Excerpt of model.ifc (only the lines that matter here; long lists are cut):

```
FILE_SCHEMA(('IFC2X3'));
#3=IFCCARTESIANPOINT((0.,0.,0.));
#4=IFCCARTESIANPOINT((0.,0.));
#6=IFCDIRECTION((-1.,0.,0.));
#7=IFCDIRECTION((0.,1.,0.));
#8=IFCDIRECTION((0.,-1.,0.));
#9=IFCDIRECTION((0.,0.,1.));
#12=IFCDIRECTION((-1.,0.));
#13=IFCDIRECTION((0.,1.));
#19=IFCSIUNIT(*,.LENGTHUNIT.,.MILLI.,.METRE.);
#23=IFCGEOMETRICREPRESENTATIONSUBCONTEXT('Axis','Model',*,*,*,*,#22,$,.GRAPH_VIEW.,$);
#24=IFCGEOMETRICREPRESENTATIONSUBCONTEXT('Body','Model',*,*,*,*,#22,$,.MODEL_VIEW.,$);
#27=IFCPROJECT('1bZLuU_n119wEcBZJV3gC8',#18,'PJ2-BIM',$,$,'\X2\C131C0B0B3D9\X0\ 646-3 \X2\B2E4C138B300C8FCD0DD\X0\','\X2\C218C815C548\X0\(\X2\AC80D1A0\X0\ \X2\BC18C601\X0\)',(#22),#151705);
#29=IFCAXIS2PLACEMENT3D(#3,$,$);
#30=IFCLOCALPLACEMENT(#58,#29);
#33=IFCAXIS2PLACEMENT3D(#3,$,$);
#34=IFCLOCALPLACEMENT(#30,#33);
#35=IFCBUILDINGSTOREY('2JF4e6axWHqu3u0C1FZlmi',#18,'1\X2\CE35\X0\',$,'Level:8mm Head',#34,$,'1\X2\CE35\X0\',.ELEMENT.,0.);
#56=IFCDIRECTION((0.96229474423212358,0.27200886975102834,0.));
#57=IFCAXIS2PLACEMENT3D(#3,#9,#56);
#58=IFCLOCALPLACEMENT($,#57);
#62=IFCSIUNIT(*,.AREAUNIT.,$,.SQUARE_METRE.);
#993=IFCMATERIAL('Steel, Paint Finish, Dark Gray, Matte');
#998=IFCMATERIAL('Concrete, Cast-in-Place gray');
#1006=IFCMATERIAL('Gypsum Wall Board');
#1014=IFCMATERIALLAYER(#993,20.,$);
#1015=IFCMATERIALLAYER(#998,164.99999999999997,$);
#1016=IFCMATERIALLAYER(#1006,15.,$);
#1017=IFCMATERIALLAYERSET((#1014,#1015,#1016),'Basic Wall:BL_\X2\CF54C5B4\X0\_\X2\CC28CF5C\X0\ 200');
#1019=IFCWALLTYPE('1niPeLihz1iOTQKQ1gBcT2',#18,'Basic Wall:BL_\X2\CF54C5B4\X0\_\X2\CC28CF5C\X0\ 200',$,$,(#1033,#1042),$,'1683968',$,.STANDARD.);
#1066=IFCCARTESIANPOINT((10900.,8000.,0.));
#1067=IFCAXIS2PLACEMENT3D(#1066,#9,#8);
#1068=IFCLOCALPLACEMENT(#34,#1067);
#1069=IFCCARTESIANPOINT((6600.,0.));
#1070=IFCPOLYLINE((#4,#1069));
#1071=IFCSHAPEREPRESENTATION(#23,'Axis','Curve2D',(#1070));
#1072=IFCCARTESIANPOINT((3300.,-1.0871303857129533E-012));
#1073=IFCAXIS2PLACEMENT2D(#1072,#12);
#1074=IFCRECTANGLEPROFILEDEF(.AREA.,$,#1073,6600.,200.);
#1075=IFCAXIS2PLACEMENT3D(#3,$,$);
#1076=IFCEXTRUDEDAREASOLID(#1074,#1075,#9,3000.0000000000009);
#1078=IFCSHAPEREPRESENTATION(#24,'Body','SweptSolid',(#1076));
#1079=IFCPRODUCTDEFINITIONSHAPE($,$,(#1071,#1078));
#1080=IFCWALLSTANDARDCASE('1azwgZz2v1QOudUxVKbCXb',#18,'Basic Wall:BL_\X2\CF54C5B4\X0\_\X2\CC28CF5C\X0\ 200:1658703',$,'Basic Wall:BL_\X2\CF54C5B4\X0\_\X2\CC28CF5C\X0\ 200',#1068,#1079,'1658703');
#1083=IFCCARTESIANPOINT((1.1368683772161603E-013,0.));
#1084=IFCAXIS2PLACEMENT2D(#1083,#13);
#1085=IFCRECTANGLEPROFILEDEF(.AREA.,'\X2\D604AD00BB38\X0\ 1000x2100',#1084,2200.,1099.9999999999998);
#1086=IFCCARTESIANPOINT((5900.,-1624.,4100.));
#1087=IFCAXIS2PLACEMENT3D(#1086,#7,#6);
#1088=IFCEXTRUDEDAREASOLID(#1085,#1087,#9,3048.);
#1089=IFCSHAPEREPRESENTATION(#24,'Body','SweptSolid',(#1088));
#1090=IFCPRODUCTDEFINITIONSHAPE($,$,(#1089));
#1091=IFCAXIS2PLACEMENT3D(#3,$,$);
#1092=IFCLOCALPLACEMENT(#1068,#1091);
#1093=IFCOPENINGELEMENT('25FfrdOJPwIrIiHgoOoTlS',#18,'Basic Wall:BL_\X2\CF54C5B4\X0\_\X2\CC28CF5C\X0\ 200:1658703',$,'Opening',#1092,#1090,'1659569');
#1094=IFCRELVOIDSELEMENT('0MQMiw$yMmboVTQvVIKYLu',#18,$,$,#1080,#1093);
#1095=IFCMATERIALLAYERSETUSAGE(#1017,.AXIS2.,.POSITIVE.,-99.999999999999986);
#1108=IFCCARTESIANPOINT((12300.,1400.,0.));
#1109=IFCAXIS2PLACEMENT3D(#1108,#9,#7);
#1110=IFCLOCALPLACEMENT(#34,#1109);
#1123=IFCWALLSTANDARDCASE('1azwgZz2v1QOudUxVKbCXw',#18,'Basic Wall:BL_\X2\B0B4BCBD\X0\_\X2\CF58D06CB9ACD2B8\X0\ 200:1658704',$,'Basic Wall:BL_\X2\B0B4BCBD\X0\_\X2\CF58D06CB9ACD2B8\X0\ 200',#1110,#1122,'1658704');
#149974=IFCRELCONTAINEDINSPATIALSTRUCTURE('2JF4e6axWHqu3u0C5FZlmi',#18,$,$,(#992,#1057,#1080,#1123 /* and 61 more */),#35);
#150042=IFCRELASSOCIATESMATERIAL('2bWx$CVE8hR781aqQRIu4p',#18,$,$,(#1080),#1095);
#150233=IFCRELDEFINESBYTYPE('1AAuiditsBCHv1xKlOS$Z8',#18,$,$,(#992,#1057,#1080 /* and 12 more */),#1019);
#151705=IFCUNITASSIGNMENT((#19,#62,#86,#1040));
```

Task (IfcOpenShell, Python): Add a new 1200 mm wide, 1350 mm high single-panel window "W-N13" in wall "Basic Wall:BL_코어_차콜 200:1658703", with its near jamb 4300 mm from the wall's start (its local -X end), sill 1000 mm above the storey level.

```python
import numpy as np
import ifcopenshell
import ifcopenshell.api.feature
import ifcopenshell.api.geometry
import ifcopenshell.api.root
import ifcopenshell.api.spatial
import ifcopenshell.api.type
import ifcopenshell.geom
import ifcopenshell.util.element
import ifcopenshell.util.placement
import ifcopenshell.util.representation
import ifcopenshell.util.shape
import ifcopenshell.util.unit

model = ifcopenshell.open("model.ifc")
unit_scale = ifcopenshell.util.unit.calculate_unit_scale(model)
settings = ifcopenshell.geom.settings()


def volume(element):
    """Net volume in cubic metres, openings subtracted."""
    shape = ifcopenshell.geom.create_shape(settings, element)
    return ifcopenshell.util.shape.get_volume(shape.geometry)


wall = model.by_guid("1azwgZz2v1QOudUxVKbCXb")
storey = ifcopenshell.util.element.get_container(wall, ifc_class="IfcBuildingStorey")
context = ifcopenshell.util.representation.get_context(model, "Model", "Body", "MODEL_VIEW")
before = volume(wall)

width, height, from_end, sill = 1.2, 1.35, 4.3, 1  # metres

# The wall runs along its own X axis, and the end named is its -X end.
wall_shape = ifcopenshell.geom.create_shape(settings, wall)
x, y, z = ifcopenshell.util.shape.get_vertices(wall_shape.geometry).T
start = x.min() + from_end
face, thickness = float(y.min()), float(y.max() - y.min())
wall_matrix = ifcopenshell.util.placement.get_local_placement(wall.ObjectPlacement)
level = ifcopenshell.util.placement.get_local_placement(storey.ObjectPlacement)[2, 3]


def in_wall(x, y):
    """Placement at x, y metres in the wall's axes, at sill height."""
    matrix = wall_matrix.copy()
    matrix[:, 3] = wall_matrix @ np.array([x / unit_scale, y / unit_scale, 0.0, 1.0])
    matrix[2, 3] = level + sill / unit_scale
    return matrix


# Opening: a box that overshoots both wall faces by 50 mm.
opening = ifcopenshell.api.root.create_entity(model, ifc_class="IfcOpeningElement")
box = ifcopenshell.api.geometry.add_wall_representation(
    model, context=context, length=width, height=height, thickness=thickness + 0.1
)
ifcopenshell.api.geometry.assign_representation(model, product=opening, representation=box)
ifcopenshell.api.geometry.edit_object_placement(model, product=opening, matrix=in_wall(start, face - 0.05), is_si=False)
ifcopenshell.api.feature.add_feature(model, feature=opening, element=wall)

window = ifcopenshell.api.root.create_entity(model, ifc_class="IfcWindow", name="W-N13")
window.OverallWidth, window.OverallHeight = width / unit_scale, height / unit_scale
body = ifcopenshell.api.geometry.add_window_representation(
    model,
    context=context,
    overall_width=window.OverallWidth,
    overall_height=window.OverallHeight,
    partition_type="SINGLE_PANEL",
)
ifcopenshell.api.geometry.assign_representation(model, product=window, representation=body)
ifcopenshell.api.spatial.assign_container(model, products=[window], relating_structure=storey)
fills = ifcopenshell.api.feature.add_filling(model, opening=opening, element=window)
fills.OwnerHistory = window.OwnerHistory  # required in IFC2X3

# IFC2X3 keeps the operation on the window style.
style = ifcopenshell.api.root.create_entity(model, ifc_class="IfcWindowStyle", name="W-N13")
style.OperationType, style.ConstructionType = "SINGLE_PANEL", "NOTDEFINED"
style.ParameterTakesPrecedence = style.Sizeable = False
ifcopenshell.api.type.assign_type(model, related_objects=[window], relating_type=style)

# Centre the window in the wall's thickness.
ifcopenshell.api.geometry.edit_object_placement(model, product=window, matrix=in_wall(start, face), is_si=False)
window_shape = ifcopenshell.geom.create_shape(settings, window)
depth = ifcopenshell.util.shape.get_vertices(window_shape.geometry)[:, 1]
offset = face + thickness / 2 - (depth.min() + depth.max()) / 2
ifcopenshell.api.geometry.edit_object_placement(model, product=window, matrix=in_wall(start, offset), is_si=False)

after = volume(wall)

print(f"wall volume {before:.3f} -> {after:.3f} m3")

model.write("model_v2.ifc")
```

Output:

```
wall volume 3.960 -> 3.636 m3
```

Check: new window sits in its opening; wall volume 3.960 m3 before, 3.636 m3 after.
